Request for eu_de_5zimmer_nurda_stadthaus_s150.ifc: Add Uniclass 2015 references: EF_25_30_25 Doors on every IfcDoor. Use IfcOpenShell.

First a look at what the model holds.

```python
import ifcopenshell

model = ifcopenshell.open("eu_de_5zimmer_nurda_stadthaus_s150.ifc")
print(model.schema)
print("classifications:", [c.Name for c in model.by_type("IfcClassification")])
for ifc_class in ("IfcDoor", "IfcRoof", "IfcStair", "IfcWall", "IfcWindow"):
    print(ifc_class, len(model.by_type(ifc_class)))
```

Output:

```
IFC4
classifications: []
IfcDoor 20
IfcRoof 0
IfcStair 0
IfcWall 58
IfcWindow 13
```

```python
import ifcopenshell
import ifcopenshell.api.classification

model = ifcopenshell.open("eu_de_5zimmer_nurda_stadthaus_s150.ifc")

system = ifcopenshell.api.classification.add_classification(model, classification="Uniclass 2015")

codes = {
    "IfcDoor": ("EF_25_30_25", "Doors"),
}
for ifc_class, (code, name) in codes.items():
    products = model.by_type(ifc_class)
    ifcopenshell.api.classification.add_reference(
        model, products=products, classification=system, identification=code, name=name
    )
    print(code, len(products))

model.write("eu_de_5zimmer_nurda_stadthaus_s150_updated.ifc")
```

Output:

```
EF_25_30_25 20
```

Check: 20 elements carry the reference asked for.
